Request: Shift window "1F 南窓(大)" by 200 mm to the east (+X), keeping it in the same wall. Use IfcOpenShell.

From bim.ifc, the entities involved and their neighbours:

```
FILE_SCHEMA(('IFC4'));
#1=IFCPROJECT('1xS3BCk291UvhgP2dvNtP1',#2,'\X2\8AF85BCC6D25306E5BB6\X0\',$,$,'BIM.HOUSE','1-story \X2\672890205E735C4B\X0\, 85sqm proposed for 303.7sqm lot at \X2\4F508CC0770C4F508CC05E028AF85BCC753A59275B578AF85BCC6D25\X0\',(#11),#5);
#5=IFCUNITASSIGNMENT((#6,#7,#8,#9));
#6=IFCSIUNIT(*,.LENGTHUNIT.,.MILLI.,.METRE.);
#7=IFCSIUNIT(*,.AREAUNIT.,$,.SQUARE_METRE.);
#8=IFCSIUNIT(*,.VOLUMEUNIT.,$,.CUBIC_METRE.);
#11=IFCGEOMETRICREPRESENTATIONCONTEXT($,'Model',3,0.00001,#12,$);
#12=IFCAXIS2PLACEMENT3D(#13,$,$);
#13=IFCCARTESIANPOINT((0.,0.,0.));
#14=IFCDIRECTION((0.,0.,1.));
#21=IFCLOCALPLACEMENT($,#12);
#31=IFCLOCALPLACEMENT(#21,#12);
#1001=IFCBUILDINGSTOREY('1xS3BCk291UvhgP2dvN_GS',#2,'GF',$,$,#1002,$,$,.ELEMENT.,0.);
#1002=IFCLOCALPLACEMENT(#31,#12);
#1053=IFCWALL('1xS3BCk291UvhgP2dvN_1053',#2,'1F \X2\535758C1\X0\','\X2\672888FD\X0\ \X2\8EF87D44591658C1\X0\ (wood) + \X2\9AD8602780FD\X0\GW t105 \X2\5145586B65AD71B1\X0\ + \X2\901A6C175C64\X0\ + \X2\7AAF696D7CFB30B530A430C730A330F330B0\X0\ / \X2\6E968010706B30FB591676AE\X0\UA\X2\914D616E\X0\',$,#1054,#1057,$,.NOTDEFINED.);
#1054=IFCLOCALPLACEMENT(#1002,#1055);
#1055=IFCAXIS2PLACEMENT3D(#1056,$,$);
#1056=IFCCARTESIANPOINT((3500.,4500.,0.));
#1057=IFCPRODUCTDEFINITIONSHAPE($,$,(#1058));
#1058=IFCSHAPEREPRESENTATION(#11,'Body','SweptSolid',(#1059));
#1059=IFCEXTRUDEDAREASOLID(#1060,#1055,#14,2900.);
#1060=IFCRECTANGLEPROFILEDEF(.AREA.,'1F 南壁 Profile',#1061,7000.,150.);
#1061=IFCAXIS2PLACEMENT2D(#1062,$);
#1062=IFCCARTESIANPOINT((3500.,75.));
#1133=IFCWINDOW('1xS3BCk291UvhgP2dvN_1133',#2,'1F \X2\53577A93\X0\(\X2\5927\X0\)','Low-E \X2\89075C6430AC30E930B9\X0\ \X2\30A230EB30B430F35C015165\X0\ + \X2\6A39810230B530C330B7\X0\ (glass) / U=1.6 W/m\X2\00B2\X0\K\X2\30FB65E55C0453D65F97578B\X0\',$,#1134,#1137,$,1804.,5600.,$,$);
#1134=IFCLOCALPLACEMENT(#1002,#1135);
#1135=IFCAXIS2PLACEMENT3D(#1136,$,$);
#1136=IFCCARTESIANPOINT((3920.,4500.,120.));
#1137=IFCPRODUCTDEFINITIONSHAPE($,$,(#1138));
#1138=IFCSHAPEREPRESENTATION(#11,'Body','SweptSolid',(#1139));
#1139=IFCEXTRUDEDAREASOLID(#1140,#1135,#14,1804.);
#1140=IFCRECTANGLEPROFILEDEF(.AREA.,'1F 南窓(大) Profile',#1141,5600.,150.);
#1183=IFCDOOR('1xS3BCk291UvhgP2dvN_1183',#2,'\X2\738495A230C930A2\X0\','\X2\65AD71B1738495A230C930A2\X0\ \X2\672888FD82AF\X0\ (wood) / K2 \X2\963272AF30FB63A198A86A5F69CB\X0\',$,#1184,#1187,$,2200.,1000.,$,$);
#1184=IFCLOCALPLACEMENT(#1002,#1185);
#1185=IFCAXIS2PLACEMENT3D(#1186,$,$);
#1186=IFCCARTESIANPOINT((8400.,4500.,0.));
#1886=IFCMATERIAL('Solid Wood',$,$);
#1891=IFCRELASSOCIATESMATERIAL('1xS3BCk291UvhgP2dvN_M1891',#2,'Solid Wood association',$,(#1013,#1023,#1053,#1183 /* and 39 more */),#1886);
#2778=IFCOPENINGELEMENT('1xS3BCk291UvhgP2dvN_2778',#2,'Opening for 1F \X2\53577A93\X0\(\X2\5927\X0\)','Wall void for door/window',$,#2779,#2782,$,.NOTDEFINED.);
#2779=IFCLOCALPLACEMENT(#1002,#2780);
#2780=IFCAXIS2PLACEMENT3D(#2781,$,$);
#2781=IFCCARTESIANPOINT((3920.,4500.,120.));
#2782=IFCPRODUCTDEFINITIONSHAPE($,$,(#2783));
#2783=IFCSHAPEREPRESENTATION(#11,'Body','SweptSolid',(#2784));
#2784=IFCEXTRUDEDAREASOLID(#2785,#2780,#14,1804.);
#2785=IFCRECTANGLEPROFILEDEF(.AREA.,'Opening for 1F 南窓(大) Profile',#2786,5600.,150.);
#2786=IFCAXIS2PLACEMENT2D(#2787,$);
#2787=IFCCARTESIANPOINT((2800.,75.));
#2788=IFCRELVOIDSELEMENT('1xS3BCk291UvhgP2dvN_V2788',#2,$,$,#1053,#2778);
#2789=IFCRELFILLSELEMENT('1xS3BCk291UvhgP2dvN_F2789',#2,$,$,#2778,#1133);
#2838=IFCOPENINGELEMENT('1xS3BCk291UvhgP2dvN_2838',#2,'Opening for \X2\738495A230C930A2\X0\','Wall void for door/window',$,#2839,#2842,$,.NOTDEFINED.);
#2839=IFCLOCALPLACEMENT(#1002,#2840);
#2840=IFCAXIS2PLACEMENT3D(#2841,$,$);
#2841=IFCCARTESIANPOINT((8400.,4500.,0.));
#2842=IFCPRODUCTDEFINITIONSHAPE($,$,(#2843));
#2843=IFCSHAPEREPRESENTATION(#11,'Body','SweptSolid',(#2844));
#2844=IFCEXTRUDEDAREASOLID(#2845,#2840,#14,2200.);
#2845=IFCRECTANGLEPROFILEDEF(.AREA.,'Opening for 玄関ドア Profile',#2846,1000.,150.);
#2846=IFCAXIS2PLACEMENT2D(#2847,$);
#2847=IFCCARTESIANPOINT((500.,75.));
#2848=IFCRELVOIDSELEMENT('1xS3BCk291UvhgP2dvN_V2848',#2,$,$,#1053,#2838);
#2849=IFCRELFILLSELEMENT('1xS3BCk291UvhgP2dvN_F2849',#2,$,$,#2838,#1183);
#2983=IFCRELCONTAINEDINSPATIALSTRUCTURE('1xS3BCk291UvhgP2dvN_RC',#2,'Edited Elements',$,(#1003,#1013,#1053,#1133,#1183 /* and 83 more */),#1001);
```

```python
import ifcopenshell
import ifcopenshell.api.geometry
import ifcopenshell.util.placement

model = ifcopenshell.open("bim.ifc")

window = model.by_id(1133)
opening = window.FillsVoids[0].RelatingOpeningElement
wall = opening.VoidsElements[0].RelatingBuildingElement

wall_matrix = ifcopenshell.util.placement.get_local_placement(wall.ObjectPlacement)
shift = wall_matrix[:3, 0] * 200.0
before = ifcopenshell.util.placement.get_local_placement(window.ObjectPlacement)[:3, 3].copy()

# The window is not placed relative to its opening, so move both.
for product in (opening, window):
    matrix = ifcopenshell.util.placement.get_local_placement(product.ObjectPlacement)
    matrix[:3, 3] += shift
    ifcopenshell.api.geometry.edit_object_placement(model, product=product, matrix=matrix, is_si=False)

after = ifcopenshell.util.placement.get_local_placement(window.ObjectPlacement)[:3, 3]
print("window moved by", (after - before).round(3) + 0.0)

model.write("bim-out.ifc")
```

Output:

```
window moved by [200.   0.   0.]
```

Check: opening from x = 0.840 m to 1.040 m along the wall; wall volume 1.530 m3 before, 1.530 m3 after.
